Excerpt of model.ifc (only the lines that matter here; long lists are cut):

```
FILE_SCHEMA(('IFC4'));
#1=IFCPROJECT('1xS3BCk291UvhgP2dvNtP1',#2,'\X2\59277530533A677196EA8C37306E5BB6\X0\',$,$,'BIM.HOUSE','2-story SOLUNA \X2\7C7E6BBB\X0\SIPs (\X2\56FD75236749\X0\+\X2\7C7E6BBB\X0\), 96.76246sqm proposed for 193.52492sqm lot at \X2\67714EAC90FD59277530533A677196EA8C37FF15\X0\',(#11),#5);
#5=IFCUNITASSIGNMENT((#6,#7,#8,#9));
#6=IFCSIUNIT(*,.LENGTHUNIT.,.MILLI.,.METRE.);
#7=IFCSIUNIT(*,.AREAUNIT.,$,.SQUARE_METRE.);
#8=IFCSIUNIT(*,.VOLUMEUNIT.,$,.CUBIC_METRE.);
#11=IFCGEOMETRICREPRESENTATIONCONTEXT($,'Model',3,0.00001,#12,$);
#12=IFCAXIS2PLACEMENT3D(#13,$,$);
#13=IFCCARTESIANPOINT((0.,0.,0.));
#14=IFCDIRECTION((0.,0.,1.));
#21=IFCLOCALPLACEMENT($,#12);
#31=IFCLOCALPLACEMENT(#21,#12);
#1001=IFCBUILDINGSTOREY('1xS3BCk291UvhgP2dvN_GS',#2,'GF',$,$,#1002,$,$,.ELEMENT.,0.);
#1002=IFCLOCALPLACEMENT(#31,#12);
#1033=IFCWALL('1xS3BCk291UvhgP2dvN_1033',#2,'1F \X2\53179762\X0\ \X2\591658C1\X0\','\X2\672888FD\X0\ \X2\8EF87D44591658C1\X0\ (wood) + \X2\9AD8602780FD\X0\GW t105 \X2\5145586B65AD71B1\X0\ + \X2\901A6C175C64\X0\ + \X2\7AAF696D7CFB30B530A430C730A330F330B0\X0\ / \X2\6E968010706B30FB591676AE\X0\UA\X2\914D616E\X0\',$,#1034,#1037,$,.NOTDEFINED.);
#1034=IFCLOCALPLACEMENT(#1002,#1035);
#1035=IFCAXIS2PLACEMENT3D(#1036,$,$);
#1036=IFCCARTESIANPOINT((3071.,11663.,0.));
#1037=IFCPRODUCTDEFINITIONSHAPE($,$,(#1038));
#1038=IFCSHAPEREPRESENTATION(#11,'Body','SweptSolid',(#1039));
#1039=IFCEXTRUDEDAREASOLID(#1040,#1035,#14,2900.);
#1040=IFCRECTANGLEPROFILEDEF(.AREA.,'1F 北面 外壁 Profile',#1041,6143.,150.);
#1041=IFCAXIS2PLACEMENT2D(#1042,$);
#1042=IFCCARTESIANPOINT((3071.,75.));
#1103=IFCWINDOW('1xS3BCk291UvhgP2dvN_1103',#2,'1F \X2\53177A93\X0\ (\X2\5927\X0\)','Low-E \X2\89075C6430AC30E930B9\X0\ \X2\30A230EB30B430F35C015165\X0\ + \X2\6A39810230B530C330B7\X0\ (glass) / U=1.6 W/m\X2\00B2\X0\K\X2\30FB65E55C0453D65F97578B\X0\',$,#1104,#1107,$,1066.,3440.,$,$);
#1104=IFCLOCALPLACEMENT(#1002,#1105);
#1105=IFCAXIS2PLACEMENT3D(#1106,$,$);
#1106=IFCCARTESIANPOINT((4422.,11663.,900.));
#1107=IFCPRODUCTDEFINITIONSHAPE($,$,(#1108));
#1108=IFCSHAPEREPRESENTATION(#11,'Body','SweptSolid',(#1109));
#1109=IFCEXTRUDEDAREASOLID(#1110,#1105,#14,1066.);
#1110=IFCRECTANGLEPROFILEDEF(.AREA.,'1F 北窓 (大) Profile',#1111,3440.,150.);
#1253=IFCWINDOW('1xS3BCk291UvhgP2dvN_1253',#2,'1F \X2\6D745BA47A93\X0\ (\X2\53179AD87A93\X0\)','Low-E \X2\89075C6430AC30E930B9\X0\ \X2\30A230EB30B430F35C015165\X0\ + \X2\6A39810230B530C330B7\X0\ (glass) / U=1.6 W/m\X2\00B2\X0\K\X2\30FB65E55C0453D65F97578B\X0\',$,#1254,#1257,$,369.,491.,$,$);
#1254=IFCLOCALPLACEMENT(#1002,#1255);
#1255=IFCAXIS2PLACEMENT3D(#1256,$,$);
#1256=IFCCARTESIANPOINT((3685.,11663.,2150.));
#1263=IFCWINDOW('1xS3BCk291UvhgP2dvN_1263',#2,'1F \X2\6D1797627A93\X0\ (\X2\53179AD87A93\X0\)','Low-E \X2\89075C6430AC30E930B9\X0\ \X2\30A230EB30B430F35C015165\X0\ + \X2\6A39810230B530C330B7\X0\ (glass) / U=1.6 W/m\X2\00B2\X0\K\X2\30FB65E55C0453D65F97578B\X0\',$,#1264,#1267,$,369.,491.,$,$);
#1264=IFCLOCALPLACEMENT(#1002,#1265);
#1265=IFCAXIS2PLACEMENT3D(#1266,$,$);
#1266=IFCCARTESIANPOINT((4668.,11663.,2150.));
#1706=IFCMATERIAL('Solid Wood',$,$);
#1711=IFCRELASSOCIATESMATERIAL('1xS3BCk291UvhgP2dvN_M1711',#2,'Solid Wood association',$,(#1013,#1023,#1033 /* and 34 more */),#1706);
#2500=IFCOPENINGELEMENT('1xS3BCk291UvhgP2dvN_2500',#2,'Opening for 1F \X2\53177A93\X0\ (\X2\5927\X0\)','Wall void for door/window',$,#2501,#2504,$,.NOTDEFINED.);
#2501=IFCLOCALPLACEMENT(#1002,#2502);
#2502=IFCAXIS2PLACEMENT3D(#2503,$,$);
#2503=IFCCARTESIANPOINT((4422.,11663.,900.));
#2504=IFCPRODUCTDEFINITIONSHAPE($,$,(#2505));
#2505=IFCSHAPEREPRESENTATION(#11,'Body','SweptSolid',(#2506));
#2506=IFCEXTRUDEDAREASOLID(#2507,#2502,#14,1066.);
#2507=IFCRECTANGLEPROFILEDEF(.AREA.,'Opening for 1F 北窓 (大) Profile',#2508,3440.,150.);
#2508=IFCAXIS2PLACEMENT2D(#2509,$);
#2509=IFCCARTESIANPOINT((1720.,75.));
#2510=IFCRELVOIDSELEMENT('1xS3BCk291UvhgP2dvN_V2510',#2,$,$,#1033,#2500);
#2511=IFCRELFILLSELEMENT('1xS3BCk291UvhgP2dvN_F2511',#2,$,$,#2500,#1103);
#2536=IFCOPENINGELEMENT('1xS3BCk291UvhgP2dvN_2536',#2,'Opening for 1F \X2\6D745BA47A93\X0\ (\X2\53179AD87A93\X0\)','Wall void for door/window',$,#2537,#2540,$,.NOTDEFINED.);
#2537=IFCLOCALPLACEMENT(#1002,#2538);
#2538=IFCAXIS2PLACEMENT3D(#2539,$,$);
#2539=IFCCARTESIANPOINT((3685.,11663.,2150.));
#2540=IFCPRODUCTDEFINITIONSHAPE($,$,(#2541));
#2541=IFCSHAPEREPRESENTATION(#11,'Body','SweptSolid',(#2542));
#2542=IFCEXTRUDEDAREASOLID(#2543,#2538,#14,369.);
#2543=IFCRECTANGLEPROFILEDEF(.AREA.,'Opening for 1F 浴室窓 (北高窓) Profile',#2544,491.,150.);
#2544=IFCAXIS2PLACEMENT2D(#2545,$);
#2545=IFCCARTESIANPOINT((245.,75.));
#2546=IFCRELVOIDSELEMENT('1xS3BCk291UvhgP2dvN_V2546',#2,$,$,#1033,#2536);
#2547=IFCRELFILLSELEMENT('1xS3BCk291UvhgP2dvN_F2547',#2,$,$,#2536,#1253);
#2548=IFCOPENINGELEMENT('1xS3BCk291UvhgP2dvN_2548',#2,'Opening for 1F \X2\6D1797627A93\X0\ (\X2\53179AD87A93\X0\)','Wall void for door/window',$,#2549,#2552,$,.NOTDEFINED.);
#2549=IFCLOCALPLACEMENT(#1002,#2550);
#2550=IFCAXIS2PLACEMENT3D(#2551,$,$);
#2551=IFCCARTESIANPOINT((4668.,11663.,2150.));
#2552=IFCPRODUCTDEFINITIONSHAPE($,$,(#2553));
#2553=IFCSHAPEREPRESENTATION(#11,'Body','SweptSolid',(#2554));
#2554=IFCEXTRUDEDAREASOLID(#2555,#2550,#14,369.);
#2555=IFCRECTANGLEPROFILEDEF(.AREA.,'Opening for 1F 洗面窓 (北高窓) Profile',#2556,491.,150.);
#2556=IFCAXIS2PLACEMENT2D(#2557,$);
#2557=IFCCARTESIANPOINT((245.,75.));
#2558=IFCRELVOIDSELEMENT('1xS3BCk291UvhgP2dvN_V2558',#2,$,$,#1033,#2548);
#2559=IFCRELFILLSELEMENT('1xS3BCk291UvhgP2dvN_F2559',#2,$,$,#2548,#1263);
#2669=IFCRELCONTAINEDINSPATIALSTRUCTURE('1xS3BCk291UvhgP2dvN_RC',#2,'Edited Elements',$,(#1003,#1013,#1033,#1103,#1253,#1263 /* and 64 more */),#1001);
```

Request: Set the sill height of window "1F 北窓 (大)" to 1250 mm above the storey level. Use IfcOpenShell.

```python
import numpy as np
import ifcopenshell
import ifcopenshell.api.geometry
import ifcopenshell.geom
import ifcopenshell.util.element
import ifcopenshell.util.placement
import ifcopenshell.util.shape
import ifcopenshell.util.unit

model = ifcopenshell.open("model.ifc")
unit_scale = ifcopenshell.util.unit.calculate_unit_scale(model)

window = model.by_guid("1xS3BCk291UvhgP2dvN_1103")
opening = window.FillsVoids[0].RelatingOpeningElement
storey = ifcopenshell.util.element.get_container(window, ifc_class="IfcBuildingStorey")
level = ifcopenshell.util.placement.get_local_placement(storey.ObjectPlacement)[2, 3]

# The opening's origin need not be at the sill, so measure its lowest point.
shape = ifcopenshell.geom.create_shape(ifcopenshell.geom.settings(), opening)
bottom = ifcopenshell.util.shape.get_shape_bottom_elevation(shape, shape.geometry) / unit_scale
dz = level + 1.25 / unit_scale - bottom

shift = np.array([0.0, 0.0, dz])
# The window is not placed relative to its opening, so move both.
for product in (opening, window):
    matrix = ifcopenshell.util.placement.get_local_placement(product.ObjectPlacement)
    matrix[:3, 3] += shift
    ifcopenshell.api.geometry.edit_object_placement(model, product=product, matrix=matrix, is_si=False)

print(f"moved by {dz * unit_scale:+.3f} m")

model.write("model_rev.ifc")
```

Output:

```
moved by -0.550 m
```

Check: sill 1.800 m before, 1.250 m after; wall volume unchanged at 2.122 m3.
